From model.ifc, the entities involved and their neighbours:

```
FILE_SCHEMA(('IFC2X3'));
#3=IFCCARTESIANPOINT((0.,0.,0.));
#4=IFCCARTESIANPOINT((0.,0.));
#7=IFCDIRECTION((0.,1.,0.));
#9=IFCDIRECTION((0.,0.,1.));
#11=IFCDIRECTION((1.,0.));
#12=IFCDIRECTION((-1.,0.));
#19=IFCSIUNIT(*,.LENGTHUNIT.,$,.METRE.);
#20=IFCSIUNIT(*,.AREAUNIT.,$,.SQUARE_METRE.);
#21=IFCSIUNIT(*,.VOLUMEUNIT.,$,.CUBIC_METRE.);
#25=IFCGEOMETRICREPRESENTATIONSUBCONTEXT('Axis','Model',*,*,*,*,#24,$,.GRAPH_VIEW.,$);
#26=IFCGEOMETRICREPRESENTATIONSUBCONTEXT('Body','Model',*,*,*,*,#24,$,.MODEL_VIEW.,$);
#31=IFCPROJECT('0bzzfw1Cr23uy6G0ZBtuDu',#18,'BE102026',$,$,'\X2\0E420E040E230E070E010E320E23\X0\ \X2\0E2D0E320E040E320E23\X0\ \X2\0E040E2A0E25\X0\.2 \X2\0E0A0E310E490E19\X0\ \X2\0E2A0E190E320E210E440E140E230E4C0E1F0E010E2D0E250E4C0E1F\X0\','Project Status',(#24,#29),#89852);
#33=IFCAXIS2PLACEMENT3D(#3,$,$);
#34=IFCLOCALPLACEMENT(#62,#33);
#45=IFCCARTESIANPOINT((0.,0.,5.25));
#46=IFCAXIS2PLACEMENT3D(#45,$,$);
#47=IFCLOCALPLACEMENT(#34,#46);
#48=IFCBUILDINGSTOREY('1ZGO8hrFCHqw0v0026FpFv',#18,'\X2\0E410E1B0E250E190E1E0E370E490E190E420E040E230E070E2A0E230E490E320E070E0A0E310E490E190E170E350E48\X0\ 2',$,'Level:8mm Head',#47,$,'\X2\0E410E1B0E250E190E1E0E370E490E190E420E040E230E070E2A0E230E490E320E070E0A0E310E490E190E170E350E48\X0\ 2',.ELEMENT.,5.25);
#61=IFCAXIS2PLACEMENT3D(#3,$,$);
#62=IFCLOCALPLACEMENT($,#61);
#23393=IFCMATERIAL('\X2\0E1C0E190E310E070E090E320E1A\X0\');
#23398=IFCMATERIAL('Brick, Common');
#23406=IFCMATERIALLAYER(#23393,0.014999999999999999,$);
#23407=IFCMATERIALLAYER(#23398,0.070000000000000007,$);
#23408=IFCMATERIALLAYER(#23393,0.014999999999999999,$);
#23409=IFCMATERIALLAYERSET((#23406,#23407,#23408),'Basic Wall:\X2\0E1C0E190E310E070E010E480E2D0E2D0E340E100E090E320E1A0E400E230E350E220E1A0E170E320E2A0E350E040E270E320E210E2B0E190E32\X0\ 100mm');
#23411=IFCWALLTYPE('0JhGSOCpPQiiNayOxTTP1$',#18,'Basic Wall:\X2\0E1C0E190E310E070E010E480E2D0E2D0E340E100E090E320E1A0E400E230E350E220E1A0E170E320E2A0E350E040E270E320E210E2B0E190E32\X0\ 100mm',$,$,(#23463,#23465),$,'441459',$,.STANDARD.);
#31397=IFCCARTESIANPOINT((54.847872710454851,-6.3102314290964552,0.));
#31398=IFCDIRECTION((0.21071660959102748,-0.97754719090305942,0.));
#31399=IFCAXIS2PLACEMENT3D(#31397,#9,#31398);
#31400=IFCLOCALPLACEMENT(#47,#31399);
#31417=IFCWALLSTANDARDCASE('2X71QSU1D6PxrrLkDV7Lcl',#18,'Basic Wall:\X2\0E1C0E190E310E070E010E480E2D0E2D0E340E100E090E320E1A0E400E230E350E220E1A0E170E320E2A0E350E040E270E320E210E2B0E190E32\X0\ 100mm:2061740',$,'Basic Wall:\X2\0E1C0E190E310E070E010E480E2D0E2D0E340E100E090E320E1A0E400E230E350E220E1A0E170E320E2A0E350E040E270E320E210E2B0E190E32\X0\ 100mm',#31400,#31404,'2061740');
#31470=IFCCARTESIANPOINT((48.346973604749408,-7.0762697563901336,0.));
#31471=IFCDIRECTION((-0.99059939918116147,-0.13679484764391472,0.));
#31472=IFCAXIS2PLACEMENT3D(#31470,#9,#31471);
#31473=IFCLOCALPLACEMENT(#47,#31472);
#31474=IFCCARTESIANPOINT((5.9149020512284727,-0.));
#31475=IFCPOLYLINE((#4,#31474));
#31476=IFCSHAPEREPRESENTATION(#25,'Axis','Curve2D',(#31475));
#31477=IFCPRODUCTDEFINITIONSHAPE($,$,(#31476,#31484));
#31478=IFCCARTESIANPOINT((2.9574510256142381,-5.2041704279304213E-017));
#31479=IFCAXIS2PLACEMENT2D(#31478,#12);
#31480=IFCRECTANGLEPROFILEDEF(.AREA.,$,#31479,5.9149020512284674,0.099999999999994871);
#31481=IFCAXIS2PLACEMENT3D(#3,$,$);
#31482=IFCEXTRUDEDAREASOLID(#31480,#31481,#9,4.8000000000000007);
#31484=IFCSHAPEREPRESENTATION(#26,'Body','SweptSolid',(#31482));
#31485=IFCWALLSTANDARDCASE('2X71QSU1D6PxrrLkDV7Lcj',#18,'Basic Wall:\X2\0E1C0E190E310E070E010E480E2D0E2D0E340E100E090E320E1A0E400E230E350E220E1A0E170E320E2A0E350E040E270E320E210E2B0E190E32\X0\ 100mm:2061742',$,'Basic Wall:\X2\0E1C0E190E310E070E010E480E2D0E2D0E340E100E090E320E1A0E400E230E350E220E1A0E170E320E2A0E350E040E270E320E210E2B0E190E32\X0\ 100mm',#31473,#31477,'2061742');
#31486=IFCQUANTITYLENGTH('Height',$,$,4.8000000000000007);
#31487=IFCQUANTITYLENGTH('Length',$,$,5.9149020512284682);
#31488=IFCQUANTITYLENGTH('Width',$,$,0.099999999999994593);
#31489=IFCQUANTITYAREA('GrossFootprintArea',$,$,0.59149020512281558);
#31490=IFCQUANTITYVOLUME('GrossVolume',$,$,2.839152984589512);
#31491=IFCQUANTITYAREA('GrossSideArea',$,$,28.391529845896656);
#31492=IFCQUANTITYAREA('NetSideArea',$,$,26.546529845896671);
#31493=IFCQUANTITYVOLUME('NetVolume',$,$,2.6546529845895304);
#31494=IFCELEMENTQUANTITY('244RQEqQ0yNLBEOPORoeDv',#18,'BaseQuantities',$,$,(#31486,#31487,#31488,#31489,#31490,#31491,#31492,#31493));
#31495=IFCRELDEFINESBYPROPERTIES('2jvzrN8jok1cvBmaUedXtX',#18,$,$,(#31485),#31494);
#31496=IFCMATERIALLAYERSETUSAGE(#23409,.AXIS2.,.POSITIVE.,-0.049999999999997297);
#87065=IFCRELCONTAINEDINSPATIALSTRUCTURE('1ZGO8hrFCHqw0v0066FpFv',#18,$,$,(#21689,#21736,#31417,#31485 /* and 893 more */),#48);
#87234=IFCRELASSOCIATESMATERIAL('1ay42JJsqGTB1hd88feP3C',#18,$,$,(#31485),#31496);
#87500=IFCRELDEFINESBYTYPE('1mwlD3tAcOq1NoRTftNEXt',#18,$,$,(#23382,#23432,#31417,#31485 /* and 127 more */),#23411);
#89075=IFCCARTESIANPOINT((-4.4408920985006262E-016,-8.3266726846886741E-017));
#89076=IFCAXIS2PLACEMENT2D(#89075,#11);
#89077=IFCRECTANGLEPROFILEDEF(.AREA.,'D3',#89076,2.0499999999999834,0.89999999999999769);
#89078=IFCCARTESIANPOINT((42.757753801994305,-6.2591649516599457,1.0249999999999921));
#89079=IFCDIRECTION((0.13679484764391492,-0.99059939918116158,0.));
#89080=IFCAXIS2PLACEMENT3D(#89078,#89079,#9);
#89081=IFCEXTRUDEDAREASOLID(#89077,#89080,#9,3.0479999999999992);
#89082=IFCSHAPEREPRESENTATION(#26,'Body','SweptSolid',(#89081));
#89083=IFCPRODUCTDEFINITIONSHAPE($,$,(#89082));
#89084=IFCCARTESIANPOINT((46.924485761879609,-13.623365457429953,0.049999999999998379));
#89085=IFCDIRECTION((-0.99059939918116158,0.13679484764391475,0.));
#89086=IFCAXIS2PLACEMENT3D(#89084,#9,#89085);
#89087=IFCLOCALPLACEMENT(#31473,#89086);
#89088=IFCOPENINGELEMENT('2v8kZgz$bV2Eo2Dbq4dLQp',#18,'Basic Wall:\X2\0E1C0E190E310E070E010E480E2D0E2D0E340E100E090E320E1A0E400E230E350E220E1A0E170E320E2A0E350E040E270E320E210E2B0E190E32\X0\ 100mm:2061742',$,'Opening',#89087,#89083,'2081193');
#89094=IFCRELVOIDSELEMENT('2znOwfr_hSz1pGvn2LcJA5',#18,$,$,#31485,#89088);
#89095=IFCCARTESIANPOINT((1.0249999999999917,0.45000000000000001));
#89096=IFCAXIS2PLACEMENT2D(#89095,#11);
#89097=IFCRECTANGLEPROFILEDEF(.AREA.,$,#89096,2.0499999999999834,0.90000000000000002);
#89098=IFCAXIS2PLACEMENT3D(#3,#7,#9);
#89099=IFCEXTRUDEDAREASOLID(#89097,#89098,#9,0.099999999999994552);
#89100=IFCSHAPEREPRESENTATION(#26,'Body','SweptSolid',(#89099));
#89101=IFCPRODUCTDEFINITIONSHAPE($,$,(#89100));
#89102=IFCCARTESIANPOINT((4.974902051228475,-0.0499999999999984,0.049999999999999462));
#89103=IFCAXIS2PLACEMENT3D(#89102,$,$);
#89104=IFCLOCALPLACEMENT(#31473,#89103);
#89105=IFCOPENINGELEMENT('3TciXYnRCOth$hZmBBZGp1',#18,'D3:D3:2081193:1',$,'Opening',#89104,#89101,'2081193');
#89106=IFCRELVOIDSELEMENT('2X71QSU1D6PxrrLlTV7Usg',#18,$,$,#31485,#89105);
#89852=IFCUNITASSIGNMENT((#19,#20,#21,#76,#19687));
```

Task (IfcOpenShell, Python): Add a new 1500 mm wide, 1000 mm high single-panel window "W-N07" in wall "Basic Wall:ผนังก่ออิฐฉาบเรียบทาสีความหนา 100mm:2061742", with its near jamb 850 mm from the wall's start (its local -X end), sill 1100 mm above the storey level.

```python
import numpy as np
import ifcopenshell
import ifcopenshell.api.feature
import ifcopenshell.api.geometry
import ifcopenshell.api.pset
import ifcopenshell.api.root
import ifcopenshell.api.spatial
import ifcopenshell.api.type
import ifcopenshell.geom
import ifcopenshell.util.element
import ifcopenshell.util.placement
import ifcopenshell.util.representation
import ifcopenshell.util.shape
import ifcopenshell.util.unit

model = ifcopenshell.open("model.ifc")
unit_scale = ifcopenshell.util.unit.calculate_unit_scale(model)
area_scale = ifcopenshell.util.unit.calculate_unit_scale(model, "AREAUNIT")
volume_scale = ifcopenshell.util.unit.calculate_unit_scale(model, "VOLUMEUNIT")
settings = ifcopenshell.geom.settings()


def volume(element):
    """Net volume in cubic metres, openings subtracted."""
    shape = ifcopenshell.geom.create_shape(settings, element)
    return ifcopenshell.util.shape.get_volume(shape.geometry)


wall = model.by_guid("2X71QSU1D6PxrrLkDV7Lcj")
storey = ifcopenshell.util.element.get_container(wall, ifc_class="IfcBuildingStorey")
context = ifcopenshell.util.representation.get_context(model, "Model", "Body", "MODEL_VIEW")
before = volume(wall)

width, height, from_end, sill = 1.5, 1, 0.85, 1.1  # metres

# The wall runs along its own X axis, and the end named is its -X end.
wall_shape = ifcopenshell.geom.create_shape(settings, wall)
x, y, z = ifcopenshell.util.shape.get_vertices(wall_shape.geometry).T
start = x.min() + from_end
face, thickness = float(y.min()), float(y.max() - y.min())
wall_matrix = ifcopenshell.util.placement.get_local_placement(wall.ObjectPlacement)
level = ifcopenshell.util.placement.get_local_placement(storey.ObjectPlacement)[2, 3]


def in_wall(x, y):
    """Placement at x, y metres in the wall's axes, at sill height."""
    matrix = wall_matrix.copy()
    matrix[:, 3] = wall_matrix @ np.array([x / unit_scale, y / unit_scale, 0.0, 1.0])
    matrix[2, 3] = level + sill / unit_scale
    return matrix


# Opening: a box that overshoots both wall faces by 50 mm.
opening = ifcopenshell.api.root.create_entity(model, ifc_class="IfcOpeningElement")
box = ifcopenshell.api.geometry.add_wall_representation(
    model, context=context, length=width, height=height, thickness=thickness + 0.1
)
ifcopenshell.api.geometry.assign_representation(model, product=opening, representation=box)
ifcopenshell.api.geometry.edit_object_placement(model, product=opening, matrix=in_wall(start, face - 0.05), is_si=False)
ifcopenshell.api.feature.add_feature(model, feature=opening, element=wall)

window = ifcopenshell.api.root.create_entity(model, ifc_class="IfcWindow", name="W-N07")
window.OverallWidth, window.OverallHeight = width / unit_scale, height / unit_scale
body = ifcopenshell.api.geometry.add_window_representation(
    model,
    context=context,
    overall_width=window.OverallWidth,
    overall_height=window.OverallHeight,
    partition_type="SINGLE_PANEL",
)
ifcopenshell.api.geometry.assign_representation(model, product=window, representation=body)
ifcopenshell.api.spatial.assign_container(model, products=[window], relating_structure=storey)
fills = ifcopenshell.api.feature.add_filling(model, opening=opening, element=window)
fills.OwnerHistory = window.OwnerHistory  # required in IFC2X3

# IFC2X3 keeps the operation on the window style.
style = ifcopenshell.api.root.create_entity(model, ifc_class="IfcWindowStyle", name="W-N07")
style.OperationType, style.ConstructionType = "SINGLE_PANEL", "NOTDEFINED"
style.ParameterTakesPrecedence = style.Sizeable = False
ifcopenshell.api.type.assign_type(model, related_objects=[window], relating_type=style)

# Centre the window in the wall's thickness.
ifcopenshell.api.geometry.edit_object_placement(model, product=window, matrix=in_wall(start, face), is_si=False)
window_shape = ifcopenshell.geom.create_shape(settings, window)
depth = ifcopenshell.util.shape.get_vertices(window_shape.geometry)[:, 1]
offset = face + thickness / 2 - (depth.min() + depth.max()) / 2
ifcopenshell.api.geometry.edit_object_placement(model, product=window, matrix=in_wall(start, offset), is_si=False)

after = volume(wall)

# Update the wall's stored quantities.
qto = model.by_id(ifcopenshell.util.element.get_pset(wall, "BaseQuantities", should_inherit=False)["id"])
ifcopenshell.api.pset.edit_qto(model, qto=qto, properties={
    "NetSideArea": after / thickness / area_scale,
    "NetVolume": after / volume_scale,
})

print(f"wall volume {before:.3f} -> {after:.3f} m3")

model.write("model-out.ifc")
```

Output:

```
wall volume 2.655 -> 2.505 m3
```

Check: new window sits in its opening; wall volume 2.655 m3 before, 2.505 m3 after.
